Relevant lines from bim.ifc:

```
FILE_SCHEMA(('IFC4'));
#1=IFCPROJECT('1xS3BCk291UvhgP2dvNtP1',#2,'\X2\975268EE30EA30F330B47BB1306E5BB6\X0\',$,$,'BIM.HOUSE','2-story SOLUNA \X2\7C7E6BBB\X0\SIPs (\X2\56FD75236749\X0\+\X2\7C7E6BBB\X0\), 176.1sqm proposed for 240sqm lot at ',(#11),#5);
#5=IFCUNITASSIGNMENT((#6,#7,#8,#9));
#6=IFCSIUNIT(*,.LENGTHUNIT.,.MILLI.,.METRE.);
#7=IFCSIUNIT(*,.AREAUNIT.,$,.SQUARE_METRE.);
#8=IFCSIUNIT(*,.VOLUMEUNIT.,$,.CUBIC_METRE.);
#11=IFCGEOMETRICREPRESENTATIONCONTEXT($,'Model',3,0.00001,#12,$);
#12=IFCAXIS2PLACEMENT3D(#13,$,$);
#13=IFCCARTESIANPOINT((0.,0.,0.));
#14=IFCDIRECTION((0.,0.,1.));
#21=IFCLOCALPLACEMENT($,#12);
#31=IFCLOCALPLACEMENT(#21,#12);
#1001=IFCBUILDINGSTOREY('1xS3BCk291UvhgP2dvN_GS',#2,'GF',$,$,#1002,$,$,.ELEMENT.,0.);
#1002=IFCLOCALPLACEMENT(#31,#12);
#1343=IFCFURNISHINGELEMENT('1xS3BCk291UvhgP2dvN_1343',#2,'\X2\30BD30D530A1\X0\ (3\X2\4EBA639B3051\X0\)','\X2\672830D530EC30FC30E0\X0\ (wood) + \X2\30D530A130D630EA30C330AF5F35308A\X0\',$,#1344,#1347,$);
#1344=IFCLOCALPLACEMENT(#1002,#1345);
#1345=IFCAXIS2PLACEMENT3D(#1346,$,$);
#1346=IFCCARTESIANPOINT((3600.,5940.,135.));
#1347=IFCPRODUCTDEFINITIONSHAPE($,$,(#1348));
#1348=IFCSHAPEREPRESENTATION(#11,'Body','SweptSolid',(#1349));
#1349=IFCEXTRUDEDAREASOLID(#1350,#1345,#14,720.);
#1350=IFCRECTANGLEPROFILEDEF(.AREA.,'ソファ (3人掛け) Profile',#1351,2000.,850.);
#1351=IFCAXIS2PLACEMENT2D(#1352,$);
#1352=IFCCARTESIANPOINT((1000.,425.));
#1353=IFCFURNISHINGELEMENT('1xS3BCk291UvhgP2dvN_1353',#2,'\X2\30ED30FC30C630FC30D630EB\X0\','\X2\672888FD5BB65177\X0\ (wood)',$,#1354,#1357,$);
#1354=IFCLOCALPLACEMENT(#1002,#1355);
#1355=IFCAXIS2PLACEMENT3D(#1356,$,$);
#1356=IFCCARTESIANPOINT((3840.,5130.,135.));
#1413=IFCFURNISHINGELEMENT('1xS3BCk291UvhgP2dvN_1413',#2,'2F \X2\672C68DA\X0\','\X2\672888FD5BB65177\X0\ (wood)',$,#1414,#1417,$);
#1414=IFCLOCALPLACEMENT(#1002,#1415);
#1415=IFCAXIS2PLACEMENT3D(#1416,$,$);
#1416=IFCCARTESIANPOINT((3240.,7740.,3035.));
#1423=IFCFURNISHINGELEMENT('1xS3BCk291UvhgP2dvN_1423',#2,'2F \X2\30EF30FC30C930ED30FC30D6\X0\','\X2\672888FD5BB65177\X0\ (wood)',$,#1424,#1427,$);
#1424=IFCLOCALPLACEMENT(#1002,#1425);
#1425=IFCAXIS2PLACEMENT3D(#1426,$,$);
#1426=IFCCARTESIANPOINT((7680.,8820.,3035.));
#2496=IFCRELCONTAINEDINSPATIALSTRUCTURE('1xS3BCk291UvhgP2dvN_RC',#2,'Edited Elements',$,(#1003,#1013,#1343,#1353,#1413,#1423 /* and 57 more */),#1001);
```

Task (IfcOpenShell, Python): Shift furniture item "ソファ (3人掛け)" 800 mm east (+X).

```python
import ifcopenshell
import ifcopenshell.api.geometry
import ifcopenshell.util.placement

model = ifcopenshell.open("bim.ifc")

item = model.by_guid("1xS3BCk291UvhgP2dvN_1343")
matrix = ifcopenshell.util.placement.get_local_placement(item.ObjectPlacement)
matrix[0, 3] += 800.0
ifcopenshell.api.geometry.edit_object_placement(model, product=item, matrix=matrix, is_si=False)

print(ifcopenshell.util.placement.get_local_placement(item.ObjectPlacement).round(3) + 0.0)

model.write("bim_edited.ifc")
```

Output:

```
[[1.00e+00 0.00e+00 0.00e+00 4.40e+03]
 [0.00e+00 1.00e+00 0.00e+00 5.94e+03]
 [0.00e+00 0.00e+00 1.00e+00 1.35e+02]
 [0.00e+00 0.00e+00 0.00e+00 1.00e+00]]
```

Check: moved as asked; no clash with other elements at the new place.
